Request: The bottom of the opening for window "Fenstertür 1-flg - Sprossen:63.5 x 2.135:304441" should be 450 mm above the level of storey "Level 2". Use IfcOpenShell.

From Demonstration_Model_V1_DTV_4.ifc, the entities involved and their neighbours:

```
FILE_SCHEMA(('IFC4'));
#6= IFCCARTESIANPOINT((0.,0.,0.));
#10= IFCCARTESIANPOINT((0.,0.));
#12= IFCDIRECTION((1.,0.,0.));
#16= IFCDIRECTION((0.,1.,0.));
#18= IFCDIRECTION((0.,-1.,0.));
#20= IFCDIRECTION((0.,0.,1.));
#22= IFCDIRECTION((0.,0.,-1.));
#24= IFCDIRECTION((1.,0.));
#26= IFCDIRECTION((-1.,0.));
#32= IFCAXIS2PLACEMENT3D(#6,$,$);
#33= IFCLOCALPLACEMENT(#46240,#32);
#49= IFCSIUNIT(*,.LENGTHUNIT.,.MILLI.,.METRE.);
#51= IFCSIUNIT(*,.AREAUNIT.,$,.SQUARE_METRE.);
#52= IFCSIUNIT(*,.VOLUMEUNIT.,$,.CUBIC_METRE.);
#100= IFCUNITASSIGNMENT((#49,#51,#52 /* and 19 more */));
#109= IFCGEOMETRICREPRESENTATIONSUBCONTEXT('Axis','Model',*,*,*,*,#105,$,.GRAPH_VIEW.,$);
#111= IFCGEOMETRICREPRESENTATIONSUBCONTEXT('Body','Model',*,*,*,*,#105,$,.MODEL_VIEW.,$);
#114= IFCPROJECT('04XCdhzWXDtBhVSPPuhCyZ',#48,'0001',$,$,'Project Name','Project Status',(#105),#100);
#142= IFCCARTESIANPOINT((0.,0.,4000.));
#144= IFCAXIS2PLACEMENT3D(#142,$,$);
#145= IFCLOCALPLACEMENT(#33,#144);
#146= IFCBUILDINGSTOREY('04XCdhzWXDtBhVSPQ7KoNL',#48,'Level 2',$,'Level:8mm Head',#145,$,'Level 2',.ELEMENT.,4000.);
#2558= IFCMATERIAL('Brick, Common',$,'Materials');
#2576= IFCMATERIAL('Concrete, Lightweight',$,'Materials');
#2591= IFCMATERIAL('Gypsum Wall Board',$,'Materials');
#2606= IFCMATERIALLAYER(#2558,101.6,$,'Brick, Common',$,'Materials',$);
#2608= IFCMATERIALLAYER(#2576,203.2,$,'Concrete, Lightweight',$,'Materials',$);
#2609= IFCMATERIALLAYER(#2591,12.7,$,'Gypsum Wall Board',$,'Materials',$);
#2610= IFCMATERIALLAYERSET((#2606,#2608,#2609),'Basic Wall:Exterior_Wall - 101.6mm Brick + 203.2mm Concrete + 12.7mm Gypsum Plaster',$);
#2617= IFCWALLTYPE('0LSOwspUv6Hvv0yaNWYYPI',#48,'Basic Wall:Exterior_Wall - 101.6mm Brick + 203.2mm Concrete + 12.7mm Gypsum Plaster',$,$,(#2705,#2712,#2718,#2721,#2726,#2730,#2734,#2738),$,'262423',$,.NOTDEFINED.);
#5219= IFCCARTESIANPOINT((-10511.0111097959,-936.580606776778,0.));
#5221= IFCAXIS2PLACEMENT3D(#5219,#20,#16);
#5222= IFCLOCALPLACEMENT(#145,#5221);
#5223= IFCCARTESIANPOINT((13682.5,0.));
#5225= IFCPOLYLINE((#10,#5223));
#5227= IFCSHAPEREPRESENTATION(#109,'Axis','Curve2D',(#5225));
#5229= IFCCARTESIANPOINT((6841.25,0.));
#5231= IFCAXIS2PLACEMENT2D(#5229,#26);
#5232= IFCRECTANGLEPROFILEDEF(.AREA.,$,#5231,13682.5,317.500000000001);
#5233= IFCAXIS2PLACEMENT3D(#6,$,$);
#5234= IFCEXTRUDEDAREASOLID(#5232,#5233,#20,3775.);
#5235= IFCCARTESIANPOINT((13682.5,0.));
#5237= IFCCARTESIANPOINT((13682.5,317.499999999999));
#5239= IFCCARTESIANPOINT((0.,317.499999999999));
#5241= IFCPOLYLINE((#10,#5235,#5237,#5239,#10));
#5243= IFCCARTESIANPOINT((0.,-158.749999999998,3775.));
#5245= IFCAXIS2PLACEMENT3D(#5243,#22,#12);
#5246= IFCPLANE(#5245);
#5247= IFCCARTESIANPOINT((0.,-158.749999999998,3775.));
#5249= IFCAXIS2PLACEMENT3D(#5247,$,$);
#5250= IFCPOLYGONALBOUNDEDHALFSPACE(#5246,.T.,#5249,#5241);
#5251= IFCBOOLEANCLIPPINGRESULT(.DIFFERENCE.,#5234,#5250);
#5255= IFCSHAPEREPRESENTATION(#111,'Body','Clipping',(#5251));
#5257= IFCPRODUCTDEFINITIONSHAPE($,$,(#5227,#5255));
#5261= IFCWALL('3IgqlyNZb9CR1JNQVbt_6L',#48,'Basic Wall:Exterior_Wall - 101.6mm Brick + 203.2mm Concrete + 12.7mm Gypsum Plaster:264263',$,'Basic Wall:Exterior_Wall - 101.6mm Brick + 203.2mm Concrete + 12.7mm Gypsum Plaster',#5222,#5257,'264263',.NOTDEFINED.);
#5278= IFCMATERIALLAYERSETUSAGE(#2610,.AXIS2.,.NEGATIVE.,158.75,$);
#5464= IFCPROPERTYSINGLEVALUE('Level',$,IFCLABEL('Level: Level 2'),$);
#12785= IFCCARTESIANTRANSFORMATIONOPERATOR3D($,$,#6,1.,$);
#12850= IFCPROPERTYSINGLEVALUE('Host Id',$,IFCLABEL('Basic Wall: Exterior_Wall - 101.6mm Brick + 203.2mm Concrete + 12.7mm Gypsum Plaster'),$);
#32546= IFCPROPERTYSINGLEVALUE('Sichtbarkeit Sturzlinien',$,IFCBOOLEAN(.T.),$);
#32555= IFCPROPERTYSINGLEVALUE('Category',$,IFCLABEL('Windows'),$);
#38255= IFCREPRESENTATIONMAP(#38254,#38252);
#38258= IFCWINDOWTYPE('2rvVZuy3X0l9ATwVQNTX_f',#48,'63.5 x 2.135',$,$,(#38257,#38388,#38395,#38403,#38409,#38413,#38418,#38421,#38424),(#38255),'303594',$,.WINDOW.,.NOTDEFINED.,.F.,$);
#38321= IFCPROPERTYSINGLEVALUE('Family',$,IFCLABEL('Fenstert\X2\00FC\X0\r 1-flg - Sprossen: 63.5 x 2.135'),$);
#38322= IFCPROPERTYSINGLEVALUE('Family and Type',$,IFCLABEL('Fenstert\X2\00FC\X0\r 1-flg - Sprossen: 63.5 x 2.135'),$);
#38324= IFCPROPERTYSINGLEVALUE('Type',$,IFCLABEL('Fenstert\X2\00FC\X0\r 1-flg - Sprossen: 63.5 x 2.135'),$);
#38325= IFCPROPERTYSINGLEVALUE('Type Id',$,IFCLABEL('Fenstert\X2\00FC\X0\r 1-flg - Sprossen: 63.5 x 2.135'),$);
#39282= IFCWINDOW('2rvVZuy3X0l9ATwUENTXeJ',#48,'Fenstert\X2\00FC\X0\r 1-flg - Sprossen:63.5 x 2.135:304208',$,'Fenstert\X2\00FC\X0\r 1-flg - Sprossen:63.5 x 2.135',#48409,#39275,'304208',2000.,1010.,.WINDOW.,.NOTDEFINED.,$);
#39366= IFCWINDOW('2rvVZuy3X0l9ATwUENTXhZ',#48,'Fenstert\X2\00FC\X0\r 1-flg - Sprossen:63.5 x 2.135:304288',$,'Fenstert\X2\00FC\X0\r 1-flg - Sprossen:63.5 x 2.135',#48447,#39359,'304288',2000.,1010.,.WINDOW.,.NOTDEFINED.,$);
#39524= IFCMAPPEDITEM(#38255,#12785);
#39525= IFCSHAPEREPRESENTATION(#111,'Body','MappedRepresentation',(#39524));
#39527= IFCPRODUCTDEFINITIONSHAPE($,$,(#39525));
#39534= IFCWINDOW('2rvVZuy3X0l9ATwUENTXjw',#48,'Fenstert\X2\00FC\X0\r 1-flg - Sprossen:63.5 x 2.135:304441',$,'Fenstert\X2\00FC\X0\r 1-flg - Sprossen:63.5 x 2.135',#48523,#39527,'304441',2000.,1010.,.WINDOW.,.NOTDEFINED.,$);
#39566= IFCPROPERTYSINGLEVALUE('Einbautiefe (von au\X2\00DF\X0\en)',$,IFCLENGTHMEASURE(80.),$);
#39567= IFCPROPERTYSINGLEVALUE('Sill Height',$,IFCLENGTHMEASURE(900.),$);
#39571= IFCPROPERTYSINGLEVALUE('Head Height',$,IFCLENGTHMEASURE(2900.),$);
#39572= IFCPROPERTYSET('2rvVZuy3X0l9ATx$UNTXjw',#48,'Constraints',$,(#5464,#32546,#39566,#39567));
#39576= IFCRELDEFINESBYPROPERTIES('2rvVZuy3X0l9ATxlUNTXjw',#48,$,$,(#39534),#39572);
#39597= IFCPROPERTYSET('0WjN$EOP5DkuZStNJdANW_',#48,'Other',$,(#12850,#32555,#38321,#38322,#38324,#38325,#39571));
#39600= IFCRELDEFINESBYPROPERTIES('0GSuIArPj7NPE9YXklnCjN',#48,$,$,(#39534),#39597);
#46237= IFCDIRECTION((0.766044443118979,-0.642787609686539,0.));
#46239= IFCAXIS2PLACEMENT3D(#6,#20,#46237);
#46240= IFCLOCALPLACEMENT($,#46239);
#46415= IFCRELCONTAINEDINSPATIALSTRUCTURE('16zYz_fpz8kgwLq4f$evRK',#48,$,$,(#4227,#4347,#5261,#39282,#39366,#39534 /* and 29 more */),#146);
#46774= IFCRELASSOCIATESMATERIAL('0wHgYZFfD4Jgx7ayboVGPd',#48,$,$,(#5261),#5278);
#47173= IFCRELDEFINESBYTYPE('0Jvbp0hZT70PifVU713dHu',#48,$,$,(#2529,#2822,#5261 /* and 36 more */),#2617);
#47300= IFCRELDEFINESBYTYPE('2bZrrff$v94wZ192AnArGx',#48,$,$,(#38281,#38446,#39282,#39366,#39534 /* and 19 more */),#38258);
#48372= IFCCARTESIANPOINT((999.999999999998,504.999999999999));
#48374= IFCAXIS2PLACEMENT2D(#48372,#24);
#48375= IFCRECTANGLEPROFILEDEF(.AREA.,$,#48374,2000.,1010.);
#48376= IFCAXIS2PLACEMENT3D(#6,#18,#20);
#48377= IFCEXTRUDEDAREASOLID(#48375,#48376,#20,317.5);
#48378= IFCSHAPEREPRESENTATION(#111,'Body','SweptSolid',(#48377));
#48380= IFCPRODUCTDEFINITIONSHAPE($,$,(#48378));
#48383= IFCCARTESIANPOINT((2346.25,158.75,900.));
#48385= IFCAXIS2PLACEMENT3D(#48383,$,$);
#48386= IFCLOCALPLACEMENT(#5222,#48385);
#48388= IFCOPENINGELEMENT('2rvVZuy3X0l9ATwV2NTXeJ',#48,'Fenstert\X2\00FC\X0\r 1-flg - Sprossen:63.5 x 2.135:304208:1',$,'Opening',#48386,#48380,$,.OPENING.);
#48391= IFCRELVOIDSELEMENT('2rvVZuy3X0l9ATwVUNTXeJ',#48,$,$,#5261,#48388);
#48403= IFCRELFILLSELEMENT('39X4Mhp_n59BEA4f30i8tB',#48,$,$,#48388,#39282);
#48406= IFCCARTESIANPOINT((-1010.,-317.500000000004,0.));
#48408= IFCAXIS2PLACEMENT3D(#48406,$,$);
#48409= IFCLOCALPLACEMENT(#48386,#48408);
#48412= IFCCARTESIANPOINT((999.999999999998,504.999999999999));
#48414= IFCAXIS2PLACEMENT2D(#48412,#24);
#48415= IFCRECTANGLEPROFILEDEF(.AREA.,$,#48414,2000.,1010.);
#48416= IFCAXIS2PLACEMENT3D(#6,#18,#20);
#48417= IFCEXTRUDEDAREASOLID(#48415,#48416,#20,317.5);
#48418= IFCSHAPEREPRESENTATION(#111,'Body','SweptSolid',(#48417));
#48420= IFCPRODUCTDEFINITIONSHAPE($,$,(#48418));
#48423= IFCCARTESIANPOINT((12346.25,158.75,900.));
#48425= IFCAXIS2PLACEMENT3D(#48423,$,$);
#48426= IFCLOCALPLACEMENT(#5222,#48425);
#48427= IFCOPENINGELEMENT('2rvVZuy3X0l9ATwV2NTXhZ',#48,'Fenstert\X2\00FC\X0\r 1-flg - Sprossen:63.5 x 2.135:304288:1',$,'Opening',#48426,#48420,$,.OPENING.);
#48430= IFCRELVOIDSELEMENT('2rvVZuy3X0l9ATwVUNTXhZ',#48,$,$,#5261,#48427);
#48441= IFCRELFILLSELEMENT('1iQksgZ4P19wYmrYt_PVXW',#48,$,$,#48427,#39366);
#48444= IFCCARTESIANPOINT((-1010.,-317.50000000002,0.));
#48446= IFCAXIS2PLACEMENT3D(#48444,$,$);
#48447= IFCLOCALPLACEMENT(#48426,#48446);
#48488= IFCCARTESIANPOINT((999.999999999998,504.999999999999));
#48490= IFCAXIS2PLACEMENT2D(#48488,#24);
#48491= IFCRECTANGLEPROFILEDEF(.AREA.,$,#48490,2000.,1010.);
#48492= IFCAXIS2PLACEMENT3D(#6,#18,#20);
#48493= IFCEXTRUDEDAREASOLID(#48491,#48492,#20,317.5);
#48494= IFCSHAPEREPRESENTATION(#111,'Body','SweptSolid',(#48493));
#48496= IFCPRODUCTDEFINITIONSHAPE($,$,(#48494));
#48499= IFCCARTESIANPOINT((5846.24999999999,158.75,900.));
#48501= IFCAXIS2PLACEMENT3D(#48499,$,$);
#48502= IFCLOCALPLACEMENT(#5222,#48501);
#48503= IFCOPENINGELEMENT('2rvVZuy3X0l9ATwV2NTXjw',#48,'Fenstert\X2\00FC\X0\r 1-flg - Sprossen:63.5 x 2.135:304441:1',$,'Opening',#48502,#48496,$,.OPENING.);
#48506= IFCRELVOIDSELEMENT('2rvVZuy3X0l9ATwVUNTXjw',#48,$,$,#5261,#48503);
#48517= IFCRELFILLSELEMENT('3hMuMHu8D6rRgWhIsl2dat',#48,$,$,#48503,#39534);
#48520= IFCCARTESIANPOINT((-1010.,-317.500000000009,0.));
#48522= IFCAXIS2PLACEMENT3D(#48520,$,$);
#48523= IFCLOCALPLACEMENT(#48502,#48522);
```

```python
import numpy as np
import ifcopenshell
import ifcopenshell.api.geometry
import ifcopenshell.api.pset
import ifcopenshell.geom
import ifcopenshell.util.element
import ifcopenshell.util.placement
import ifcopenshell.util.shape
import ifcopenshell.util.unit

model = ifcopenshell.open("Demonstration_Model_V1_DTV_4.ifc")
unit_scale = ifcopenshell.util.unit.calculate_unit_scale(model)

window = model.by_guid("2rvVZuy3X0l9ATwUENTXjw")
opening = window.FillsVoids[0].RelatingOpeningElement
storey = ifcopenshell.util.element.get_container(window, ifc_class="IfcBuildingStorey")
level = ifcopenshell.util.placement.get_local_placement(storey.ObjectPlacement)[2, 3]

# The opening's origin need not be at the sill, so measure its lowest point.
shape = ifcopenshell.geom.create_shape(ifcopenshell.geom.settings(), opening)
bottom = ifcopenshell.util.shape.get_shape_bottom_elevation(shape, shape.geometry) / unit_scale
dz = level + 450.0 - bottom

shift = np.array([0.0, 0.0, dz])
# The window is placed relative to its opening, so it follows when the opening moves.
matrix = ifcopenshell.util.placement.get_local_placement(opening.ObjectPlacement)
matrix[:3, 3] += shift
ifcopenshell.api.geometry.edit_object_placement(
    model, product=opening, matrix=matrix, is_si=False, should_transform_children=True
)

# Keep the stored heights in step.
pset = model.by_id(ifcopenshell.util.element.get_pset(window, "Constraints", should_inherit=False)["id"])
ifcopenshell.api.pset.edit_pset(model, pset=pset, properties={
    "Sill Height": model.create_entity("IfcLengthMeasure", ifcopenshell.util.element.get_pset(window, "Constraints", "Sill Height") + dz),
})
pset = model.by_id(ifcopenshell.util.element.get_pset(window, "Other", should_inherit=False)["id"])
ifcopenshell.api.pset.edit_pset(model, pset=pset, properties={
    "Head Height": model.create_entity("IfcLengthMeasure", ifcopenshell.util.element.get_pset(window, "Other", "Head Height") + dz),
})

print(f"moved by {dz * unit_scale:+.3f} m")

model.write("Demonstration_Model_V1_DTV_4_updated.ifc")
```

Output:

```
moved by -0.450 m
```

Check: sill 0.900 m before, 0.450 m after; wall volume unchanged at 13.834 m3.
